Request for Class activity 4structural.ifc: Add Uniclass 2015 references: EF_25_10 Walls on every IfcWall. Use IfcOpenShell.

First a look at what the model holds.

```python
import ifcopenshell

model = ifcopenshell.open("Class activity 4structural.ifc")
print(model.schema)
print("classifications:", [c.Name for c in model.by_type("IfcClassification")])
for ifc_class in ("IfcDoor", "IfcRoof", "IfcStair", "IfcWall", "IfcWindow"):
    print(ifc_class, len(model.by_type(ifc_class)))
```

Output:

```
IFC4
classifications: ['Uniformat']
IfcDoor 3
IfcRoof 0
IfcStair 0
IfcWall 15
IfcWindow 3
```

```python
import ifcopenshell
import ifcopenshell.api.classification

model = ifcopenshell.open("Class activity 4structural.ifc")

system = ifcopenshell.api.classification.add_classification(model, classification="Uniclass 2015")

codes = {
    "IfcWall": ("EF_25_10", "Walls"),
}
for ifc_class, (code, name) in codes.items():
    products = model.by_type(ifc_class)
    ifcopenshell.api.classification.add_reference(
        model, products=products, classification=system, identification=code, name=name
    )
    print(code, len(products))

model.write("Class activity 4structural_updated.ifc")
```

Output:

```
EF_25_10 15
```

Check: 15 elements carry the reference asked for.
